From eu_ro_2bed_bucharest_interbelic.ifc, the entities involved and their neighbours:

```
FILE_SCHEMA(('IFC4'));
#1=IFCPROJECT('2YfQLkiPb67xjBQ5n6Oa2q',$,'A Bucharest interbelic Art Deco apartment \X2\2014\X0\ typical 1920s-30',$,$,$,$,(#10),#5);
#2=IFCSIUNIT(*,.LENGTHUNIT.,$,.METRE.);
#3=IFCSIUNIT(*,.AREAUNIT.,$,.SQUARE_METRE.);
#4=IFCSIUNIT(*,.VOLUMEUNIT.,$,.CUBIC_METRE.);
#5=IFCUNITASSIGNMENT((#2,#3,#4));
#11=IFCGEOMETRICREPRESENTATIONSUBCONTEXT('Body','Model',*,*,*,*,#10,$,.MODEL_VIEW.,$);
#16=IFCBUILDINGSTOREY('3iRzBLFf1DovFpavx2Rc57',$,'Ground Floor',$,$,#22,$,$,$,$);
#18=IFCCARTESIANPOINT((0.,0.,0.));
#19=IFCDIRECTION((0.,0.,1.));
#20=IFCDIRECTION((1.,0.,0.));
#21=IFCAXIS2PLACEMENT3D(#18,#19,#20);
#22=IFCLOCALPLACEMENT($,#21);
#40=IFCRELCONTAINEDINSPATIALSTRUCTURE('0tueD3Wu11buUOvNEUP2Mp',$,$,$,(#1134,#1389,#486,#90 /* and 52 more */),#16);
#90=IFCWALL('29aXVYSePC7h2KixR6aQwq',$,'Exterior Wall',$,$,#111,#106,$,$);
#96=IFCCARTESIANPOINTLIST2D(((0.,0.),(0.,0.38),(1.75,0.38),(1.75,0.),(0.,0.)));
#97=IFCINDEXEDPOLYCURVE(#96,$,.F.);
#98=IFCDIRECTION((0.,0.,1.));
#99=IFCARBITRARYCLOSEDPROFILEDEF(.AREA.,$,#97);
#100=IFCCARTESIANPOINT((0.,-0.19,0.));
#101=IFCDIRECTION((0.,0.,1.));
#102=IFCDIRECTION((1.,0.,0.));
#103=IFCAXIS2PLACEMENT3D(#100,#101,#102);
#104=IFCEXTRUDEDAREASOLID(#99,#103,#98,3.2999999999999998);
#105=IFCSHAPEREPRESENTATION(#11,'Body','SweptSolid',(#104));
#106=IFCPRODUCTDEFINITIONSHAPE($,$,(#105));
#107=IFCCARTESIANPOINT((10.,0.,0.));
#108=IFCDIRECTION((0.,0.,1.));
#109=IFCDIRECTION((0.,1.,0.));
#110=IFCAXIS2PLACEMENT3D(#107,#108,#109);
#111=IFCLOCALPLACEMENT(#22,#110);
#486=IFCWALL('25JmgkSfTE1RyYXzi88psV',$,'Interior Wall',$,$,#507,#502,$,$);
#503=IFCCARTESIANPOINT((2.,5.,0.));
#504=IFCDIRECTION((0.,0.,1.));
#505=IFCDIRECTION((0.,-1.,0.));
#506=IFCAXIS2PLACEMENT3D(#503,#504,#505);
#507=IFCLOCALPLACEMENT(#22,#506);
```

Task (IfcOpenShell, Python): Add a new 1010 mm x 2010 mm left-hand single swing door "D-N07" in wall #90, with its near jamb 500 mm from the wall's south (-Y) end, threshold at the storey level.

```python
import numpy as np
import ifcopenshell
import ifcopenshell.api.feature
import ifcopenshell.api.geometry
import ifcopenshell.api.root
import ifcopenshell.api.spatial
import ifcopenshell.geom
import ifcopenshell.util.element
import ifcopenshell.util.placement
import ifcopenshell.util.representation
import ifcopenshell.util.shape
import ifcopenshell.util.unit

model = ifcopenshell.open("eu_ro_2bed_bucharest_interbelic.ifc")
unit_scale = ifcopenshell.util.unit.calculate_unit_scale(model)
settings = ifcopenshell.geom.settings()


def volume(element):
    """Net volume in cubic metres, openings subtracted."""
    shape = ifcopenshell.geom.create_shape(settings, element)
    return ifcopenshell.util.shape.get_volume(shape.geometry)


wall = model.by_guid("29aXVYSePC7h2KixR6aQwq")
storey = ifcopenshell.util.element.get_container(wall, ifc_class="IfcBuildingStorey")
context = ifcopenshell.util.representation.get_context(model, "Model", "Body", "MODEL_VIEW")
before = volume(wall)

width, height, from_end, sill = 1.01, 2.01, 0.5, 0.0  # metres

# The wall runs along its own X axis, and the end named is its -X end.
wall_shape = ifcopenshell.geom.create_shape(settings, wall)
x, y, z = ifcopenshell.util.shape.get_vertices(wall_shape.geometry).T
start = x.min() + from_end
face, thickness = float(y.min()), float(y.max() - y.min())
wall_matrix = ifcopenshell.util.placement.get_local_placement(wall.ObjectPlacement)
level = ifcopenshell.util.placement.get_local_placement(storey.ObjectPlacement)[2, 3]


def in_wall(x, y):
    """Placement at x, y metres in the wall's axes, at sill height."""
    matrix = wall_matrix.copy()
    matrix[:, 3] = wall_matrix @ np.array([x / unit_scale, y / unit_scale, 0.0, 1.0])
    matrix[2, 3] = level + sill / unit_scale
    return matrix


# Opening: a box that overshoots both wall faces by 50 mm.
opening = ifcopenshell.api.root.create_entity(model, ifc_class="IfcOpeningElement", predefined_type="OPENING")
box = ifcopenshell.api.geometry.add_wall_representation(
    model, context=context, length=width, height=height, thickness=thickness + 0.1
)
ifcopenshell.api.geometry.assign_representation(model, product=opening, representation=box)
ifcopenshell.api.geometry.edit_object_placement(model, product=opening, matrix=in_wall(start, face - 0.05), is_si=False)
ifcopenshell.api.feature.add_feature(model, feature=opening, element=wall)

door = ifcopenshell.api.root.create_entity(model, ifc_class="IfcDoor", name="D-N07", predefined_type="DOOR")
door.OverallWidth, door.OverallHeight = width / unit_scale, height / unit_scale
door.OperationType = "SINGLE_SWING_LEFT"
body = ifcopenshell.api.geometry.add_door_representation(
    model,
    context=context,
    overall_width=door.OverallWidth,
    overall_height=door.OverallHeight,
    operation_type="SINGLE_SWING_LEFT",
    lining_properties={"LiningDepth": thickness / unit_scale, "ThresholdDepth": thickness / unit_scale},
)
ifcopenshell.api.geometry.assign_representation(model, product=door, representation=body)
ifcopenshell.api.spatial.assign_container(model, products=[door], relating_structure=storey)
ifcopenshell.api.feature.add_filling(model, opening=opening, element=door)

# The lining spans the wall, so the door starts at the wall face.
ifcopenshell.api.geometry.edit_object_placement(model, product=door, matrix=in_wall(start, face), is_si=False)

after = volume(wall)

print(f"wall volume {before:.3f} -> {after:.3f} m3")

model.write("eu_ro_2bed_bucharest_interbelic_v2.ifc")
```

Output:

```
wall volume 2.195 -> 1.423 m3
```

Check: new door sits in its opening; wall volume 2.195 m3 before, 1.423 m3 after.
